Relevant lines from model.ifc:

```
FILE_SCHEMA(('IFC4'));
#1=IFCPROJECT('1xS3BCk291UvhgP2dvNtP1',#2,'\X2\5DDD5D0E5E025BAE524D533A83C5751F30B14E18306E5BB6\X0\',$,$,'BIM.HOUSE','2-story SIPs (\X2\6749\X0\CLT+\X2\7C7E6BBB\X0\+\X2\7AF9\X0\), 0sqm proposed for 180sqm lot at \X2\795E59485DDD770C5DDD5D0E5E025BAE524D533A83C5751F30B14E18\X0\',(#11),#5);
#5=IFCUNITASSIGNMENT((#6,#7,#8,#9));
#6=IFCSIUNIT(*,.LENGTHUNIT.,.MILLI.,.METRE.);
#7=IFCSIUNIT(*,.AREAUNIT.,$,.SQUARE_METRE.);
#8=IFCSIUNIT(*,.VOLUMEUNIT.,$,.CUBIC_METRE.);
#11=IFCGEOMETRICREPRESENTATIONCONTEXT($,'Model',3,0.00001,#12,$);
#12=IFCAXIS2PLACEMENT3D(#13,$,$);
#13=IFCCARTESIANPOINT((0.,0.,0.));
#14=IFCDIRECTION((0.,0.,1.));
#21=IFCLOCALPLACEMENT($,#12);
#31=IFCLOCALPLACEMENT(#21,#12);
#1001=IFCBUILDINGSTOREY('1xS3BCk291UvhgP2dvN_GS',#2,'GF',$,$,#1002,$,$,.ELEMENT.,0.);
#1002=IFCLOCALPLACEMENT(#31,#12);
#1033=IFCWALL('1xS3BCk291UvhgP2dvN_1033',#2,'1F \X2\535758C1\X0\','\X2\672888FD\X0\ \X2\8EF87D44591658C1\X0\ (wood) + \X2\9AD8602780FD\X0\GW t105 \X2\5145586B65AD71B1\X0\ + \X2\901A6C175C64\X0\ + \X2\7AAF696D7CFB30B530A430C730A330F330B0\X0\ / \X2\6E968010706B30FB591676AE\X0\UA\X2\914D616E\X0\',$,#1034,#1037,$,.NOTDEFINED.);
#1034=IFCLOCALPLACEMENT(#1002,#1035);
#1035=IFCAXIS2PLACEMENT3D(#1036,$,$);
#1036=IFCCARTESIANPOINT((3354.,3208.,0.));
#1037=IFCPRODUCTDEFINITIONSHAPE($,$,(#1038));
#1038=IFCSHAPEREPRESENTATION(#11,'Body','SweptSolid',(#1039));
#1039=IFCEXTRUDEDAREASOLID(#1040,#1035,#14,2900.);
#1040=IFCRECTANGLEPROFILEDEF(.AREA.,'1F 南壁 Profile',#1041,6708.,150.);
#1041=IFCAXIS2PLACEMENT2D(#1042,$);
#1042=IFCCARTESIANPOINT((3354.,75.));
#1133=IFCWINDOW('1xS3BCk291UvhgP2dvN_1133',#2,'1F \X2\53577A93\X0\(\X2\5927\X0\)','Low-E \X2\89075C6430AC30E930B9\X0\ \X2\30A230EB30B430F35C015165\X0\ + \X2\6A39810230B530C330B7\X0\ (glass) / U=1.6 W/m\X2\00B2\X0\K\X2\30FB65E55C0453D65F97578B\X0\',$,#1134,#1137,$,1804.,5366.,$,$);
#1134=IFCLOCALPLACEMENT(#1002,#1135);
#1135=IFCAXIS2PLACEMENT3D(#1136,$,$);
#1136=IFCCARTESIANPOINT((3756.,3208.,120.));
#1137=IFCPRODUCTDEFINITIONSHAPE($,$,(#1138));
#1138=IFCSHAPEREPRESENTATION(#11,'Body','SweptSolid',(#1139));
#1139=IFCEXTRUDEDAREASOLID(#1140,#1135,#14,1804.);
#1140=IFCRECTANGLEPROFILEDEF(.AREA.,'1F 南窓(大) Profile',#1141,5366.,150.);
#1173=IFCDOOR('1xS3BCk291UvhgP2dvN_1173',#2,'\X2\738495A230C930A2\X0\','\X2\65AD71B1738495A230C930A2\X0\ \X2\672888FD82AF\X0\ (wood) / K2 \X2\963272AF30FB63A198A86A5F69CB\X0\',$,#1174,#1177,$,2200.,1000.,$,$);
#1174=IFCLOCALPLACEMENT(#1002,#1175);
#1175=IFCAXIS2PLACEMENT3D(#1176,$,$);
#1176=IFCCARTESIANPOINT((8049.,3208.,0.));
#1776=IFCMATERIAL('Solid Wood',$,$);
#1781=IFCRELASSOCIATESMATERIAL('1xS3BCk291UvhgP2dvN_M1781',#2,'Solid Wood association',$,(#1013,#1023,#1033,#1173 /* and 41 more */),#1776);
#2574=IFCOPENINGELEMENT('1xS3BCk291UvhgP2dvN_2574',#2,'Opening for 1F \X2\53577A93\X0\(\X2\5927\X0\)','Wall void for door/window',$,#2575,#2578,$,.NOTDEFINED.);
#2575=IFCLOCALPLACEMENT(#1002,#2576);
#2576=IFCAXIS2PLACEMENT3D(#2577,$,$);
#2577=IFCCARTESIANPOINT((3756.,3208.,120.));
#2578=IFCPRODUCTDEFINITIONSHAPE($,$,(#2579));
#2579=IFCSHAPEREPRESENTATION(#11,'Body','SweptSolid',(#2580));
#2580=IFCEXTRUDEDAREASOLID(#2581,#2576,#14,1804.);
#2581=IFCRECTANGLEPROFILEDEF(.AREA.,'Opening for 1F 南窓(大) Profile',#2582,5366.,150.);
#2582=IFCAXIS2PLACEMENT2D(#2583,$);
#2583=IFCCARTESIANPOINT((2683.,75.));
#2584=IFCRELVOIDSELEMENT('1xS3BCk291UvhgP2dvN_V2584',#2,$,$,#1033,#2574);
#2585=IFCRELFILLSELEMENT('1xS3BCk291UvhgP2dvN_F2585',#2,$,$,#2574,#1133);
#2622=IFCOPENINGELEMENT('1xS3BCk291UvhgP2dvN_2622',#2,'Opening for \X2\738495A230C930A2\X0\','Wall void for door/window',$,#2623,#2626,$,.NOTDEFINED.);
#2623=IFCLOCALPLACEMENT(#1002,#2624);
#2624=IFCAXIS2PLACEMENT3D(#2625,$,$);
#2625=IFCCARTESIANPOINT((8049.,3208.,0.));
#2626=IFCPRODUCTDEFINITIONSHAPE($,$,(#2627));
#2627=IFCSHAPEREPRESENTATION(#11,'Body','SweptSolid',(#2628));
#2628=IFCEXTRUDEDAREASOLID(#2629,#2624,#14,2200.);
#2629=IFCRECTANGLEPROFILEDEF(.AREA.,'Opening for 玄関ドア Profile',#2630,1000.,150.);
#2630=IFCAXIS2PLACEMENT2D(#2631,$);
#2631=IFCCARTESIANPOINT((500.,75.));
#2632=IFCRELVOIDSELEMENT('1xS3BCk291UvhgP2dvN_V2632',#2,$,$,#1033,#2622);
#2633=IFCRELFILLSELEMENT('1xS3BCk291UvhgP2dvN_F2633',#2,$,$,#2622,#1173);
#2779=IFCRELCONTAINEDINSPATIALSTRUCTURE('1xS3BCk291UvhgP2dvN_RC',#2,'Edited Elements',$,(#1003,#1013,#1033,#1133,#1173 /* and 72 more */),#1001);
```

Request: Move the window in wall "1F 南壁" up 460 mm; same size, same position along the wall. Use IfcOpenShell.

```python
import numpy as np
import ifcopenshell
import ifcopenshell.api.geometry
import ifcopenshell.util.placement
import ifcopenshell.util.unit

model = ifcopenshell.open("model.ifc")
unit_scale = ifcopenshell.util.unit.calculate_unit_scale(model)

window = model.by_guid("1xS3BCk291UvhgP2dvN_1133")
opening = window.FillsVoids[0].RelatingOpeningElement
dz = 460.0

shift = np.array([0.0, 0.0, dz])
# The window is not placed relative to its opening, so move both.
for product in (opening, window):
    matrix = ifcopenshell.util.placement.get_local_placement(product.ObjectPlacement)
    matrix[:3, 3] += shift
    ifcopenshell.api.geometry.edit_object_placement(model, product=product, matrix=matrix, is_si=False)

print(f"moved by {dz * unit_scale:+.3f} m")

model.write("model_rev.ifc")
```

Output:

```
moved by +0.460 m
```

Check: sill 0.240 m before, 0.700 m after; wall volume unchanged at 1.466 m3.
